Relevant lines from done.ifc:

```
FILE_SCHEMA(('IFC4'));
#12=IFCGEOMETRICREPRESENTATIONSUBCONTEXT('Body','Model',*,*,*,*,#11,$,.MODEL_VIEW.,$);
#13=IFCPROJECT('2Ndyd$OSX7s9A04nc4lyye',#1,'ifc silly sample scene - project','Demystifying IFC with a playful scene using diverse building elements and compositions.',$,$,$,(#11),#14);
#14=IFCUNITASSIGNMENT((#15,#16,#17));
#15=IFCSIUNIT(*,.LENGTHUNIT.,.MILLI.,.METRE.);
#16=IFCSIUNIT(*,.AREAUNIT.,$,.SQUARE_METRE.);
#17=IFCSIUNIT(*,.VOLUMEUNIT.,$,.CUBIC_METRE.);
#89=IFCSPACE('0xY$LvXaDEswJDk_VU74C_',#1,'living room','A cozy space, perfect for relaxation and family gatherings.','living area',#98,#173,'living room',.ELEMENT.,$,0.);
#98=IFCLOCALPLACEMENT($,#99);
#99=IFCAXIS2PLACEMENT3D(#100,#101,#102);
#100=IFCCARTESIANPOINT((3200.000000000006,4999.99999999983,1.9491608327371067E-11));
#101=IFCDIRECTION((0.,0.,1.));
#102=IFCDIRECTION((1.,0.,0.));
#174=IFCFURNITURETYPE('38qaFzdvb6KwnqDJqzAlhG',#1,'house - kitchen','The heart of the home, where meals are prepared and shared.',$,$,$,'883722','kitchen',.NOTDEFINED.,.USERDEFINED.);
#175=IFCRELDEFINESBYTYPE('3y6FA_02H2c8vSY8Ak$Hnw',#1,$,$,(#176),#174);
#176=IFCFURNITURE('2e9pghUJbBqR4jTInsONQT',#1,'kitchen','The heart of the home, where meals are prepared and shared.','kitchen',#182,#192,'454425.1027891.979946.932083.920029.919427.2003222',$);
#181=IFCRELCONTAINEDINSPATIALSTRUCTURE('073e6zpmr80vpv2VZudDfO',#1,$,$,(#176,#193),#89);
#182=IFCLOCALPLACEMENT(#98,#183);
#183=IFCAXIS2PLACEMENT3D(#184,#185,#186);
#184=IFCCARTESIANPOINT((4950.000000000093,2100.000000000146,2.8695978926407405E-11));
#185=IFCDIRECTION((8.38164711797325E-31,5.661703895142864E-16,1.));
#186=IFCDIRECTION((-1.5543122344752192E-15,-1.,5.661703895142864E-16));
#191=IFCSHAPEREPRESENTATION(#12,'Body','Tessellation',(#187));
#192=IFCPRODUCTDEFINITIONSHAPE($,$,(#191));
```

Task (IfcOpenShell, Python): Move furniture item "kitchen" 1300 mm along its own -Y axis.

```python
import ifcopenshell
import ifcopenshell.api.geometry
import ifcopenshell.util.placement
import ifcopenshell.util.unit

model = ifcopenshell.open("done.ifc")
unit_scale = ifcopenshell.util.unit.calculate_unit_scale(model)

item = model.by_guid("2e9pghUJbBqR4jTInsONQT")
matrix = ifcopenshell.util.placement.get_local_placement(item.ObjectPlacement)
matrix[:3, 3] -= matrix[:3, 1] * 1.3 / unit_scale
ifcopenshell.api.geometry.edit_object_placement(model, product=item, matrix=matrix, is_si=False)

print(ifcopenshell.util.placement.get_local_placement(item.ObjectPlacement).round(3) + 0.0)

model.write("done_updated.ifc")
```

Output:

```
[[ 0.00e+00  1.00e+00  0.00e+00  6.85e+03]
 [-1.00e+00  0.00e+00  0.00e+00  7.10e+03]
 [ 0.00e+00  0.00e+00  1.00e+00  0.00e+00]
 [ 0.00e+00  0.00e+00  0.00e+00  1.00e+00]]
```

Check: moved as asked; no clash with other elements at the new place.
